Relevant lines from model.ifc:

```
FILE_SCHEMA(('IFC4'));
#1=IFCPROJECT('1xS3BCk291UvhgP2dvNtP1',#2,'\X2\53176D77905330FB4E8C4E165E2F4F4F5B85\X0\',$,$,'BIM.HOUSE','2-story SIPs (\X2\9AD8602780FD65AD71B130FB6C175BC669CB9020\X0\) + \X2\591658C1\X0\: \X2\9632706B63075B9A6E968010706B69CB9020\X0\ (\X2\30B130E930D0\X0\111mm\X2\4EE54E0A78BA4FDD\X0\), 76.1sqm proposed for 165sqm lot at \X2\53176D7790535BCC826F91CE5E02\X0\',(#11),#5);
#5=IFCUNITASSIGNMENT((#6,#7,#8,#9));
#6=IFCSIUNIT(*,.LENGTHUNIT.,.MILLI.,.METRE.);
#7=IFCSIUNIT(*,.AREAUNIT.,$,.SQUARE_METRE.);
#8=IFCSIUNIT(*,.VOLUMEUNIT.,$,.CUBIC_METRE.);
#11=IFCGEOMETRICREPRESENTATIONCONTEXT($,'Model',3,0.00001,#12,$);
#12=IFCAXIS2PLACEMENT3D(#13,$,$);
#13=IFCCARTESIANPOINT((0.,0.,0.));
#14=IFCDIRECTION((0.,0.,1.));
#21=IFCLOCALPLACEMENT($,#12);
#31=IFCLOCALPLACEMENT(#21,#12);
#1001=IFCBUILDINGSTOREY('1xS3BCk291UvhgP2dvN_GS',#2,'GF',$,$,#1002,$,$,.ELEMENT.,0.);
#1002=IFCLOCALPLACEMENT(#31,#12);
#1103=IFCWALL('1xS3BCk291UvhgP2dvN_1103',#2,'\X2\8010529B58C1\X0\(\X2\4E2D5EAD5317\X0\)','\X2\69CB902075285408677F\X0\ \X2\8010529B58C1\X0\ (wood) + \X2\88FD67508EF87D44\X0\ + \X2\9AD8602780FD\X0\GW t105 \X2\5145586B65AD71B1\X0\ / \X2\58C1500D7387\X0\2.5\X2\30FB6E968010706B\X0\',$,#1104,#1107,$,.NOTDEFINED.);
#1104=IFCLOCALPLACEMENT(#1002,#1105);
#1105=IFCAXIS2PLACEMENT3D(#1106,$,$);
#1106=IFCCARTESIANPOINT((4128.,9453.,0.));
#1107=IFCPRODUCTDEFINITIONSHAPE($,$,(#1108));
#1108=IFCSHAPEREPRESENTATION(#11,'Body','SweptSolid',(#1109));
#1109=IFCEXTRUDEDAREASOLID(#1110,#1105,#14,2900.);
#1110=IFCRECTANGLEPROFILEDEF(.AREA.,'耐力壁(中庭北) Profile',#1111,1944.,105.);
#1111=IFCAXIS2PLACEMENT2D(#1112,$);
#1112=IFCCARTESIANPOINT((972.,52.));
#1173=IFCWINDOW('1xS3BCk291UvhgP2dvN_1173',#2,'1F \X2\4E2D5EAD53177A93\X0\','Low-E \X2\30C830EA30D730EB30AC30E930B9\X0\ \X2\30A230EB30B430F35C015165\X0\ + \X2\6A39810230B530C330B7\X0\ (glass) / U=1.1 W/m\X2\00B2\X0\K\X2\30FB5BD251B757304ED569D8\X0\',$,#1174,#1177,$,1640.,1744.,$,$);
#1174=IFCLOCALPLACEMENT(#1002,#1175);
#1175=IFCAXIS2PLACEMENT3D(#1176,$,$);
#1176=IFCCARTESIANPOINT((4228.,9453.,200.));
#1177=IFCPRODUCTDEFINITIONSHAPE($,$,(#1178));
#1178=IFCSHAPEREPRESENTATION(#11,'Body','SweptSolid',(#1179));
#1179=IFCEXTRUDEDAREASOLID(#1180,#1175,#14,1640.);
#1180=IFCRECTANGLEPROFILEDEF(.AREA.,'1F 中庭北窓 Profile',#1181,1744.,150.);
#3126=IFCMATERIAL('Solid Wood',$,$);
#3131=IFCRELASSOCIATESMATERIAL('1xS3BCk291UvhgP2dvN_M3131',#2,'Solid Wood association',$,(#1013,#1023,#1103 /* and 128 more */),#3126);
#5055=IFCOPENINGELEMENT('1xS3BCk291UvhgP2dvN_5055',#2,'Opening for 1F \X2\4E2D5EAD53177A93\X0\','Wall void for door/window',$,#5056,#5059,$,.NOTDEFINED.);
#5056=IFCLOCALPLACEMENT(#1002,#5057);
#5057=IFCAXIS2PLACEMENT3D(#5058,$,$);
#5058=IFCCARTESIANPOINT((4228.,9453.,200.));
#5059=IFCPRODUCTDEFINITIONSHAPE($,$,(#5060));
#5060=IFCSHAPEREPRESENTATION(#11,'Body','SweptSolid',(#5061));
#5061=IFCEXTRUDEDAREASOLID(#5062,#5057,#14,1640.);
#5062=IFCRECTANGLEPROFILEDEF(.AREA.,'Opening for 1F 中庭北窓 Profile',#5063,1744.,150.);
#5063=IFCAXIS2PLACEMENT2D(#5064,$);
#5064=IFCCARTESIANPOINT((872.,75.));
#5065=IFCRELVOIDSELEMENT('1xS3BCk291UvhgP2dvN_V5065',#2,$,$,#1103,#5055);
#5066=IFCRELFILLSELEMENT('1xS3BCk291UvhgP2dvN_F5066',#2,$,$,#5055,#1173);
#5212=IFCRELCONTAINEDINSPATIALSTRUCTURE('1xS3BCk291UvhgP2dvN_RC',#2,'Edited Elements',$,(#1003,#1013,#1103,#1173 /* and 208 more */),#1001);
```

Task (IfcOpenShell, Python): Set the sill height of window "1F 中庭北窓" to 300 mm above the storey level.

```python
import numpy as np
import ifcopenshell
import ifcopenshell.api.geometry
import ifcopenshell.geom
import ifcopenshell.util.element
import ifcopenshell.util.placement
import ifcopenshell.util.shape
import ifcopenshell.util.unit

model = ifcopenshell.open("model.ifc")
unit_scale = ifcopenshell.util.unit.calculate_unit_scale(model)

window = model.by_id(1173)
opening = window.FillsVoids[0].RelatingOpeningElement
storey = ifcopenshell.util.element.get_container(window, ifc_class="IfcBuildingStorey")
level = ifcopenshell.util.placement.get_local_placement(storey.ObjectPlacement)[2, 3]

# The opening's origin need not be at the sill, so measure its lowest point.
shape = ifcopenshell.geom.create_shape(ifcopenshell.geom.settings(), opening)
bottom = ifcopenshell.util.shape.get_shape_bottom_elevation(shape, shape.geometry) / unit_scale
dz = level + 0.3 / unit_scale - bottom

shift = np.array([0.0, 0.0, dz])
# The window is not placed relative to its opening, so move both.
for product in (opening, window):
    matrix = ifcopenshell.util.placement.get_local_placement(product.ObjectPlacement)
    matrix[:3, 3] += shift
    ifcopenshell.api.geometry.edit_object_placement(model, product=product, matrix=matrix, is_si=False)

print(f"moved by {dz * unit_scale:+.3f} m")

model.write("model-out.ifc")
```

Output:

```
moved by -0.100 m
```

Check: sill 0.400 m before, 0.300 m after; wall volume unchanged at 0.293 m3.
